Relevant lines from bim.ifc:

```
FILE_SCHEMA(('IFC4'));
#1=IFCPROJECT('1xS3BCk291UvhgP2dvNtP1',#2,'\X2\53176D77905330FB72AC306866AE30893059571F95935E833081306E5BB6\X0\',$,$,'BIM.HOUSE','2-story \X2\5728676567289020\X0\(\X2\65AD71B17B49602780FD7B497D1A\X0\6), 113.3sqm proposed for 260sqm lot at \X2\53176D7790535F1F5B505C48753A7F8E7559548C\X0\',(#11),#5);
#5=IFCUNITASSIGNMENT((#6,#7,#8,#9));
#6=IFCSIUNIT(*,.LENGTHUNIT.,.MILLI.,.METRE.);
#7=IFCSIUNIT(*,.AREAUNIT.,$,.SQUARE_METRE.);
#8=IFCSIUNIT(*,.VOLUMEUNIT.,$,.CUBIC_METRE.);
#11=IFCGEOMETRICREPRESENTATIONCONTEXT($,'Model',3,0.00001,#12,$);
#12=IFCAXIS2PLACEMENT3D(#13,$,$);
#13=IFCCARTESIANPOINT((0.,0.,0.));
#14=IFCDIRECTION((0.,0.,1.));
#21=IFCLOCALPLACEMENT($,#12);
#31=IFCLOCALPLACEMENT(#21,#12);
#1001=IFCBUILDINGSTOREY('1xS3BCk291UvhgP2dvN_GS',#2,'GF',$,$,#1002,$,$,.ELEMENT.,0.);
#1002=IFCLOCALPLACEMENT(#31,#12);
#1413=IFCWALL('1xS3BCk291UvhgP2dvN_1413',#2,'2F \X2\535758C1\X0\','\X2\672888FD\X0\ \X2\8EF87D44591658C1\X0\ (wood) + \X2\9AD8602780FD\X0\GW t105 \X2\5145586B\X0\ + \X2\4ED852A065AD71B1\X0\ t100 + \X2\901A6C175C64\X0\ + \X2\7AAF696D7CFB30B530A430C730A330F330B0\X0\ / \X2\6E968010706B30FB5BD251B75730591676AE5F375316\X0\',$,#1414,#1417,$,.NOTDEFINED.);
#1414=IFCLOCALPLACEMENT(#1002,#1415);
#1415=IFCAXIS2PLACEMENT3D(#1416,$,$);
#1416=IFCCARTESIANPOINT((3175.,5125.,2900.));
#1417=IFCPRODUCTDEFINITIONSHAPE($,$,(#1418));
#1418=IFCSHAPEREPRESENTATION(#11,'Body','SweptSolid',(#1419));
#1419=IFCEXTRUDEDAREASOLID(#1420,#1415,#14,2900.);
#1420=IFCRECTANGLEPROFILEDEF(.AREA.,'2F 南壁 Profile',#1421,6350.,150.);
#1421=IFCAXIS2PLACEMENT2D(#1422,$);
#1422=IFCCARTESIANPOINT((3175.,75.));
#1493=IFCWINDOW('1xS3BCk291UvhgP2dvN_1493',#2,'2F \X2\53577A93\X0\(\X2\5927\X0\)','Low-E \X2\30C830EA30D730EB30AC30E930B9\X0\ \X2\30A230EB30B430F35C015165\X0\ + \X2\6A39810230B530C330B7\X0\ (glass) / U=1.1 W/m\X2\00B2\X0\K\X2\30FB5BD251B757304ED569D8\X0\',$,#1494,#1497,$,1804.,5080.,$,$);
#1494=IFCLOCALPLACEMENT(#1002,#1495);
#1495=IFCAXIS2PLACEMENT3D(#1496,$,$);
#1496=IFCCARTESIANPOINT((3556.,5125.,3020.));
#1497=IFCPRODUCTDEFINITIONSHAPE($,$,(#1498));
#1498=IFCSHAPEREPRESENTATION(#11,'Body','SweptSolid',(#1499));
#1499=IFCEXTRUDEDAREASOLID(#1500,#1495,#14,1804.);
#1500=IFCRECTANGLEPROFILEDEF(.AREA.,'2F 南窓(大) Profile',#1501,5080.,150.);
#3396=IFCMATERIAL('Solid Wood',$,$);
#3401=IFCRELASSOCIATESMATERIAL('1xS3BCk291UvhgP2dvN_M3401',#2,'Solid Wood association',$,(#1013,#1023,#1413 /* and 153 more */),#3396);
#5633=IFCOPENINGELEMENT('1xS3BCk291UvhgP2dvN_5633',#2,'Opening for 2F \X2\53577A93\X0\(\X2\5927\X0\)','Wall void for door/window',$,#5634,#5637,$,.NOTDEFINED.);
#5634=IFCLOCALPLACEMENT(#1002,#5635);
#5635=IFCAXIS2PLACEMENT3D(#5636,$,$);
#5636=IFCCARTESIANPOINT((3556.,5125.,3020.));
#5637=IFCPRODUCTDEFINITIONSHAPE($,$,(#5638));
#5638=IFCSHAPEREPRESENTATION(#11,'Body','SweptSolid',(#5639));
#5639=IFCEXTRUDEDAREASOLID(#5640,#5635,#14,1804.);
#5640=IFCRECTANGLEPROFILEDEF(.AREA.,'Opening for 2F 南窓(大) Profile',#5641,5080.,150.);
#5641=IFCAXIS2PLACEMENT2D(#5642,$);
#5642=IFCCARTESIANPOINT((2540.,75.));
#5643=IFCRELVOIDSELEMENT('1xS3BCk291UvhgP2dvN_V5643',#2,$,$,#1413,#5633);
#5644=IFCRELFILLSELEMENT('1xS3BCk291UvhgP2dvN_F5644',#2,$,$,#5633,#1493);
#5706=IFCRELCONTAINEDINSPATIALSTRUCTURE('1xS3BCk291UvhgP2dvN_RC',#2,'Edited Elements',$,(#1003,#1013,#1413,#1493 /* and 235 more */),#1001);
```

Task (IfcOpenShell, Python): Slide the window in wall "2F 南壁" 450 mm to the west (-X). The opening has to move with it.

```python
import ifcopenshell
import ifcopenshell.api.geometry
import ifcopenshell.util.placement

model = ifcopenshell.open("bim.ifc")

window = model.by_guid("1xS3BCk291UvhgP2dvN_1493")
opening = window.FillsVoids[0].RelatingOpeningElement
wall = opening.VoidsElements[0].RelatingBuildingElement

wall_matrix = ifcopenshell.util.placement.get_local_placement(wall.ObjectPlacement)
shift = wall_matrix[:3, 0] * -450.0
before = ifcopenshell.util.placement.get_local_placement(window.ObjectPlacement)[:3, 3].copy()

# The window is not placed relative to its opening, so move both.
for product in (opening, window):
    matrix = ifcopenshell.util.placement.get_local_placement(product.ObjectPlacement)
    matrix[:3, 3] += shift
    ifcopenshell.api.geometry.edit_object_placement(model, product=product, matrix=matrix, is_si=False)

after = ifcopenshell.util.placement.get_local_placement(window.ObjectPlacement)[:3, 3]
print("window moved by", (after - before).round(3) + 0.0)

model.write("bim_v2.ifc")
```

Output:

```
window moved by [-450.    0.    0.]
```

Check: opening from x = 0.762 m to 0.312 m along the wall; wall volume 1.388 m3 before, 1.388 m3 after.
